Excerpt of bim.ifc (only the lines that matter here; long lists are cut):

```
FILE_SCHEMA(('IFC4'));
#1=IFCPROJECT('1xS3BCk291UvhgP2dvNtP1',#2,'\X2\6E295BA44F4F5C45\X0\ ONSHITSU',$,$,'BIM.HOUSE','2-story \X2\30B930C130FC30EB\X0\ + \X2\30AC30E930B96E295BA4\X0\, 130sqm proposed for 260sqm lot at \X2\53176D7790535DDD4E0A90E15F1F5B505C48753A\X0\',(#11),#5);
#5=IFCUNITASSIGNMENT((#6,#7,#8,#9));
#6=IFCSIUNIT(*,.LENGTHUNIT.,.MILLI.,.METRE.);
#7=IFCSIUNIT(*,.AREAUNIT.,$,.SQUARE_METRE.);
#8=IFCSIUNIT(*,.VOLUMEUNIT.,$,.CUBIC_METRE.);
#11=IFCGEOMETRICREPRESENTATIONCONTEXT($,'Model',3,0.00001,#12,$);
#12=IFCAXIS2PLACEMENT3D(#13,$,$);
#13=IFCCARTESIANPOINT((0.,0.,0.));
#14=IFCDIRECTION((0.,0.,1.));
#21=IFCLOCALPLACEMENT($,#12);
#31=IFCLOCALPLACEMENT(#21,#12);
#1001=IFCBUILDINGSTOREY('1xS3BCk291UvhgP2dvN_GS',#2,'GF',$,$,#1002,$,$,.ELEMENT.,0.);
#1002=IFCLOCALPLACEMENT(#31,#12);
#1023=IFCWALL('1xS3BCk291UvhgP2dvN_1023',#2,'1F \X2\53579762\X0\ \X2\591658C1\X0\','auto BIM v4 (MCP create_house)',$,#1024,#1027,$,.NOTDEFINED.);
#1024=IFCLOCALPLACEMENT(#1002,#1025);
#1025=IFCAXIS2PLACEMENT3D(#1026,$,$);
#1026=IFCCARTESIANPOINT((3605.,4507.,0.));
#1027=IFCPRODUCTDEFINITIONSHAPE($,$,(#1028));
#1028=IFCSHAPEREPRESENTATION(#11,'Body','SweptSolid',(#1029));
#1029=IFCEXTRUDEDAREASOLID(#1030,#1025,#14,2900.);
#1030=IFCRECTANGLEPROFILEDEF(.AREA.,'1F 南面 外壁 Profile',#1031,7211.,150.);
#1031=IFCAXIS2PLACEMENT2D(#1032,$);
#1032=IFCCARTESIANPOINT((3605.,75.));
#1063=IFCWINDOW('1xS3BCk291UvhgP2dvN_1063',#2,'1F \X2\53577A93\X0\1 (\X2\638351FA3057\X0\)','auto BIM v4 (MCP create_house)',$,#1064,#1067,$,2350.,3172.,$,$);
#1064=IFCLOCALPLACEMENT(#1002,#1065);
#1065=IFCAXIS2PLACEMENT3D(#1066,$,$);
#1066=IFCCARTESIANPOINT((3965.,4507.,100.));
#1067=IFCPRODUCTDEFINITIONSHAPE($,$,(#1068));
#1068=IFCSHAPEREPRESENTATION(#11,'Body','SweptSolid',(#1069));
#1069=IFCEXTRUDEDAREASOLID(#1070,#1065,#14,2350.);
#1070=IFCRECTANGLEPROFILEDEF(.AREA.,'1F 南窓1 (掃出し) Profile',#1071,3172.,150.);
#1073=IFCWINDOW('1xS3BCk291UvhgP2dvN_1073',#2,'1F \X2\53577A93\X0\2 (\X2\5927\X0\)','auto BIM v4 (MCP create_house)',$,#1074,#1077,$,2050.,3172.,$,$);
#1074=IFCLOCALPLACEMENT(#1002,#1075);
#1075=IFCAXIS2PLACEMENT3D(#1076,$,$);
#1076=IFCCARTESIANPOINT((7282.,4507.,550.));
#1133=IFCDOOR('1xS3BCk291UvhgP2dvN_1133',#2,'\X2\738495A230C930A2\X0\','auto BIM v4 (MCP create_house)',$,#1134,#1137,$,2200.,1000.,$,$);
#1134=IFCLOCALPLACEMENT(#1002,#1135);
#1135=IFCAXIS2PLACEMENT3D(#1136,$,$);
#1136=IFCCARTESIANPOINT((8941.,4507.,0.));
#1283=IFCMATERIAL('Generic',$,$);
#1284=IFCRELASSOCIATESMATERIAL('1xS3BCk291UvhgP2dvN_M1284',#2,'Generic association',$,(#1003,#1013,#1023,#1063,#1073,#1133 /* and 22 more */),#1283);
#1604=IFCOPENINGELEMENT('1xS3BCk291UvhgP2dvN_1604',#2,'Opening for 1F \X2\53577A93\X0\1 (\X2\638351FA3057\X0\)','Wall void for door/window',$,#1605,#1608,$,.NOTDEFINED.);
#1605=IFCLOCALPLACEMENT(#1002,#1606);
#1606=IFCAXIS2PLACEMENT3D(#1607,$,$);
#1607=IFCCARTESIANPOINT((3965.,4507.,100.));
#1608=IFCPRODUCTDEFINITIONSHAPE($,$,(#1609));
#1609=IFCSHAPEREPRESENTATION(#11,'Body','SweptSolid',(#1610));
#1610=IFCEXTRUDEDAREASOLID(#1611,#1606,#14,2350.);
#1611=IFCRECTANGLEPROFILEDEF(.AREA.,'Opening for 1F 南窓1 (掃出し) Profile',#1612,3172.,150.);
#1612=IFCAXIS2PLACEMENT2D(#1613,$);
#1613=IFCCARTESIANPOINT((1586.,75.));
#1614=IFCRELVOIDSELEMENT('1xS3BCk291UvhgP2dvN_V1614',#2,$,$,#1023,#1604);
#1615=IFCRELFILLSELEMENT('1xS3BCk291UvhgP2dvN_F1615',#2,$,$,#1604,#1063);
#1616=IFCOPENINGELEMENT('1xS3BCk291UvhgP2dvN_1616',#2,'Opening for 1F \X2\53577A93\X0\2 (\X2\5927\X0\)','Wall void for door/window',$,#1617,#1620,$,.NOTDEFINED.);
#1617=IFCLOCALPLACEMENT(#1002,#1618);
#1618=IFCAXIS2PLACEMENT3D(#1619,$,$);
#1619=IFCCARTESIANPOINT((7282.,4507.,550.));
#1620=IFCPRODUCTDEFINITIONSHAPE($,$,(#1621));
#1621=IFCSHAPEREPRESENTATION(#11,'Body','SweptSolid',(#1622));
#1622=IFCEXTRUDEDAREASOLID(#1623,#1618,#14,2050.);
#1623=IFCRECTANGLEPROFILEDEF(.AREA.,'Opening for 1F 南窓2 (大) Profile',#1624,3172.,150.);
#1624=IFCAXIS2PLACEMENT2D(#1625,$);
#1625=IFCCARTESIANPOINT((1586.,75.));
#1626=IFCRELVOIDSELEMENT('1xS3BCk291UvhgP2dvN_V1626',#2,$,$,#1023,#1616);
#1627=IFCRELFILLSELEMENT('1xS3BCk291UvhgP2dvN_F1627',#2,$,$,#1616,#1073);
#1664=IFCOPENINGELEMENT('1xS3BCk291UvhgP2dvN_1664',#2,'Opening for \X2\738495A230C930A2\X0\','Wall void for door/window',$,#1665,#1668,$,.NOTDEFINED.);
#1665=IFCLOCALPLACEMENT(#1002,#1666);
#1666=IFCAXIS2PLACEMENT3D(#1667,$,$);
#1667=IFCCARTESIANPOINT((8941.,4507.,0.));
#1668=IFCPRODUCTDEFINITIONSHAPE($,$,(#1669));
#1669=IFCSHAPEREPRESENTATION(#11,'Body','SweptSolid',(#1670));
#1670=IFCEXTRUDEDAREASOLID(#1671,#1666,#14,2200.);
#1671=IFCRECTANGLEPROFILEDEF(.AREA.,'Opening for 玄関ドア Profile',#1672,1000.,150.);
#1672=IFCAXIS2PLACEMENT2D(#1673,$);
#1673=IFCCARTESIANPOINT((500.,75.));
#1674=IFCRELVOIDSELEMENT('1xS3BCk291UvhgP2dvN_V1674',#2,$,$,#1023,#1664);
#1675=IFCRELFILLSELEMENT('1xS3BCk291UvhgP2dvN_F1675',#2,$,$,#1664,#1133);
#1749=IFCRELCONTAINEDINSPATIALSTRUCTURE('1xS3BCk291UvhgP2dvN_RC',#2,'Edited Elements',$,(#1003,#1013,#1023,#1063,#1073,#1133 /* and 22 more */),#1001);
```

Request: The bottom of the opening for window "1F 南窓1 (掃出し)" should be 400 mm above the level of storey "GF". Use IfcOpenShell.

```python
import numpy as np
import ifcopenshell
import ifcopenshell.api.geometry
import ifcopenshell.geom
import ifcopenshell.util.element
import ifcopenshell.util.placement
import ifcopenshell.util.shape
import ifcopenshell.util.unit

model = ifcopenshell.open("bim.ifc")
unit_scale = ifcopenshell.util.unit.calculate_unit_scale(model)

window = model.by_id(1063)
opening = window.FillsVoids[0].RelatingOpeningElement
storey = ifcopenshell.util.element.get_container(window, ifc_class="IfcBuildingStorey")
level = ifcopenshell.util.placement.get_local_placement(storey.ObjectPlacement)[2, 3]

# The opening's origin need not be at the sill, so measure its lowest point.
shape = ifcopenshell.geom.create_shape(ifcopenshell.geom.settings(), opening)
bottom = ifcopenshell.util.shape.get_shape_bottom_elevation(shape, shape.geometry) / unit_scale
dz = level + 0.4 / unit_scale - bottom

shift = np.array([0.0, 0.0, dz])
# The window is not placed relative to its opening, so move both.
for product in (opening, window):
    matrix = ifcopenshell.util.placement.get_local_placement(product.ObjectPlacement)
    matrix[:3, 3] += shift
    ifcopenshell.api.geometry.edit_object_placement(model, product=product, matrix=matrix, is_si=False)

print(f"moved by {dz * unit_scale:+.3f} m")

model.write("bim-out.ifc")
```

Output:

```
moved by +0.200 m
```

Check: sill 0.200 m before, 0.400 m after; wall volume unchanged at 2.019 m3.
